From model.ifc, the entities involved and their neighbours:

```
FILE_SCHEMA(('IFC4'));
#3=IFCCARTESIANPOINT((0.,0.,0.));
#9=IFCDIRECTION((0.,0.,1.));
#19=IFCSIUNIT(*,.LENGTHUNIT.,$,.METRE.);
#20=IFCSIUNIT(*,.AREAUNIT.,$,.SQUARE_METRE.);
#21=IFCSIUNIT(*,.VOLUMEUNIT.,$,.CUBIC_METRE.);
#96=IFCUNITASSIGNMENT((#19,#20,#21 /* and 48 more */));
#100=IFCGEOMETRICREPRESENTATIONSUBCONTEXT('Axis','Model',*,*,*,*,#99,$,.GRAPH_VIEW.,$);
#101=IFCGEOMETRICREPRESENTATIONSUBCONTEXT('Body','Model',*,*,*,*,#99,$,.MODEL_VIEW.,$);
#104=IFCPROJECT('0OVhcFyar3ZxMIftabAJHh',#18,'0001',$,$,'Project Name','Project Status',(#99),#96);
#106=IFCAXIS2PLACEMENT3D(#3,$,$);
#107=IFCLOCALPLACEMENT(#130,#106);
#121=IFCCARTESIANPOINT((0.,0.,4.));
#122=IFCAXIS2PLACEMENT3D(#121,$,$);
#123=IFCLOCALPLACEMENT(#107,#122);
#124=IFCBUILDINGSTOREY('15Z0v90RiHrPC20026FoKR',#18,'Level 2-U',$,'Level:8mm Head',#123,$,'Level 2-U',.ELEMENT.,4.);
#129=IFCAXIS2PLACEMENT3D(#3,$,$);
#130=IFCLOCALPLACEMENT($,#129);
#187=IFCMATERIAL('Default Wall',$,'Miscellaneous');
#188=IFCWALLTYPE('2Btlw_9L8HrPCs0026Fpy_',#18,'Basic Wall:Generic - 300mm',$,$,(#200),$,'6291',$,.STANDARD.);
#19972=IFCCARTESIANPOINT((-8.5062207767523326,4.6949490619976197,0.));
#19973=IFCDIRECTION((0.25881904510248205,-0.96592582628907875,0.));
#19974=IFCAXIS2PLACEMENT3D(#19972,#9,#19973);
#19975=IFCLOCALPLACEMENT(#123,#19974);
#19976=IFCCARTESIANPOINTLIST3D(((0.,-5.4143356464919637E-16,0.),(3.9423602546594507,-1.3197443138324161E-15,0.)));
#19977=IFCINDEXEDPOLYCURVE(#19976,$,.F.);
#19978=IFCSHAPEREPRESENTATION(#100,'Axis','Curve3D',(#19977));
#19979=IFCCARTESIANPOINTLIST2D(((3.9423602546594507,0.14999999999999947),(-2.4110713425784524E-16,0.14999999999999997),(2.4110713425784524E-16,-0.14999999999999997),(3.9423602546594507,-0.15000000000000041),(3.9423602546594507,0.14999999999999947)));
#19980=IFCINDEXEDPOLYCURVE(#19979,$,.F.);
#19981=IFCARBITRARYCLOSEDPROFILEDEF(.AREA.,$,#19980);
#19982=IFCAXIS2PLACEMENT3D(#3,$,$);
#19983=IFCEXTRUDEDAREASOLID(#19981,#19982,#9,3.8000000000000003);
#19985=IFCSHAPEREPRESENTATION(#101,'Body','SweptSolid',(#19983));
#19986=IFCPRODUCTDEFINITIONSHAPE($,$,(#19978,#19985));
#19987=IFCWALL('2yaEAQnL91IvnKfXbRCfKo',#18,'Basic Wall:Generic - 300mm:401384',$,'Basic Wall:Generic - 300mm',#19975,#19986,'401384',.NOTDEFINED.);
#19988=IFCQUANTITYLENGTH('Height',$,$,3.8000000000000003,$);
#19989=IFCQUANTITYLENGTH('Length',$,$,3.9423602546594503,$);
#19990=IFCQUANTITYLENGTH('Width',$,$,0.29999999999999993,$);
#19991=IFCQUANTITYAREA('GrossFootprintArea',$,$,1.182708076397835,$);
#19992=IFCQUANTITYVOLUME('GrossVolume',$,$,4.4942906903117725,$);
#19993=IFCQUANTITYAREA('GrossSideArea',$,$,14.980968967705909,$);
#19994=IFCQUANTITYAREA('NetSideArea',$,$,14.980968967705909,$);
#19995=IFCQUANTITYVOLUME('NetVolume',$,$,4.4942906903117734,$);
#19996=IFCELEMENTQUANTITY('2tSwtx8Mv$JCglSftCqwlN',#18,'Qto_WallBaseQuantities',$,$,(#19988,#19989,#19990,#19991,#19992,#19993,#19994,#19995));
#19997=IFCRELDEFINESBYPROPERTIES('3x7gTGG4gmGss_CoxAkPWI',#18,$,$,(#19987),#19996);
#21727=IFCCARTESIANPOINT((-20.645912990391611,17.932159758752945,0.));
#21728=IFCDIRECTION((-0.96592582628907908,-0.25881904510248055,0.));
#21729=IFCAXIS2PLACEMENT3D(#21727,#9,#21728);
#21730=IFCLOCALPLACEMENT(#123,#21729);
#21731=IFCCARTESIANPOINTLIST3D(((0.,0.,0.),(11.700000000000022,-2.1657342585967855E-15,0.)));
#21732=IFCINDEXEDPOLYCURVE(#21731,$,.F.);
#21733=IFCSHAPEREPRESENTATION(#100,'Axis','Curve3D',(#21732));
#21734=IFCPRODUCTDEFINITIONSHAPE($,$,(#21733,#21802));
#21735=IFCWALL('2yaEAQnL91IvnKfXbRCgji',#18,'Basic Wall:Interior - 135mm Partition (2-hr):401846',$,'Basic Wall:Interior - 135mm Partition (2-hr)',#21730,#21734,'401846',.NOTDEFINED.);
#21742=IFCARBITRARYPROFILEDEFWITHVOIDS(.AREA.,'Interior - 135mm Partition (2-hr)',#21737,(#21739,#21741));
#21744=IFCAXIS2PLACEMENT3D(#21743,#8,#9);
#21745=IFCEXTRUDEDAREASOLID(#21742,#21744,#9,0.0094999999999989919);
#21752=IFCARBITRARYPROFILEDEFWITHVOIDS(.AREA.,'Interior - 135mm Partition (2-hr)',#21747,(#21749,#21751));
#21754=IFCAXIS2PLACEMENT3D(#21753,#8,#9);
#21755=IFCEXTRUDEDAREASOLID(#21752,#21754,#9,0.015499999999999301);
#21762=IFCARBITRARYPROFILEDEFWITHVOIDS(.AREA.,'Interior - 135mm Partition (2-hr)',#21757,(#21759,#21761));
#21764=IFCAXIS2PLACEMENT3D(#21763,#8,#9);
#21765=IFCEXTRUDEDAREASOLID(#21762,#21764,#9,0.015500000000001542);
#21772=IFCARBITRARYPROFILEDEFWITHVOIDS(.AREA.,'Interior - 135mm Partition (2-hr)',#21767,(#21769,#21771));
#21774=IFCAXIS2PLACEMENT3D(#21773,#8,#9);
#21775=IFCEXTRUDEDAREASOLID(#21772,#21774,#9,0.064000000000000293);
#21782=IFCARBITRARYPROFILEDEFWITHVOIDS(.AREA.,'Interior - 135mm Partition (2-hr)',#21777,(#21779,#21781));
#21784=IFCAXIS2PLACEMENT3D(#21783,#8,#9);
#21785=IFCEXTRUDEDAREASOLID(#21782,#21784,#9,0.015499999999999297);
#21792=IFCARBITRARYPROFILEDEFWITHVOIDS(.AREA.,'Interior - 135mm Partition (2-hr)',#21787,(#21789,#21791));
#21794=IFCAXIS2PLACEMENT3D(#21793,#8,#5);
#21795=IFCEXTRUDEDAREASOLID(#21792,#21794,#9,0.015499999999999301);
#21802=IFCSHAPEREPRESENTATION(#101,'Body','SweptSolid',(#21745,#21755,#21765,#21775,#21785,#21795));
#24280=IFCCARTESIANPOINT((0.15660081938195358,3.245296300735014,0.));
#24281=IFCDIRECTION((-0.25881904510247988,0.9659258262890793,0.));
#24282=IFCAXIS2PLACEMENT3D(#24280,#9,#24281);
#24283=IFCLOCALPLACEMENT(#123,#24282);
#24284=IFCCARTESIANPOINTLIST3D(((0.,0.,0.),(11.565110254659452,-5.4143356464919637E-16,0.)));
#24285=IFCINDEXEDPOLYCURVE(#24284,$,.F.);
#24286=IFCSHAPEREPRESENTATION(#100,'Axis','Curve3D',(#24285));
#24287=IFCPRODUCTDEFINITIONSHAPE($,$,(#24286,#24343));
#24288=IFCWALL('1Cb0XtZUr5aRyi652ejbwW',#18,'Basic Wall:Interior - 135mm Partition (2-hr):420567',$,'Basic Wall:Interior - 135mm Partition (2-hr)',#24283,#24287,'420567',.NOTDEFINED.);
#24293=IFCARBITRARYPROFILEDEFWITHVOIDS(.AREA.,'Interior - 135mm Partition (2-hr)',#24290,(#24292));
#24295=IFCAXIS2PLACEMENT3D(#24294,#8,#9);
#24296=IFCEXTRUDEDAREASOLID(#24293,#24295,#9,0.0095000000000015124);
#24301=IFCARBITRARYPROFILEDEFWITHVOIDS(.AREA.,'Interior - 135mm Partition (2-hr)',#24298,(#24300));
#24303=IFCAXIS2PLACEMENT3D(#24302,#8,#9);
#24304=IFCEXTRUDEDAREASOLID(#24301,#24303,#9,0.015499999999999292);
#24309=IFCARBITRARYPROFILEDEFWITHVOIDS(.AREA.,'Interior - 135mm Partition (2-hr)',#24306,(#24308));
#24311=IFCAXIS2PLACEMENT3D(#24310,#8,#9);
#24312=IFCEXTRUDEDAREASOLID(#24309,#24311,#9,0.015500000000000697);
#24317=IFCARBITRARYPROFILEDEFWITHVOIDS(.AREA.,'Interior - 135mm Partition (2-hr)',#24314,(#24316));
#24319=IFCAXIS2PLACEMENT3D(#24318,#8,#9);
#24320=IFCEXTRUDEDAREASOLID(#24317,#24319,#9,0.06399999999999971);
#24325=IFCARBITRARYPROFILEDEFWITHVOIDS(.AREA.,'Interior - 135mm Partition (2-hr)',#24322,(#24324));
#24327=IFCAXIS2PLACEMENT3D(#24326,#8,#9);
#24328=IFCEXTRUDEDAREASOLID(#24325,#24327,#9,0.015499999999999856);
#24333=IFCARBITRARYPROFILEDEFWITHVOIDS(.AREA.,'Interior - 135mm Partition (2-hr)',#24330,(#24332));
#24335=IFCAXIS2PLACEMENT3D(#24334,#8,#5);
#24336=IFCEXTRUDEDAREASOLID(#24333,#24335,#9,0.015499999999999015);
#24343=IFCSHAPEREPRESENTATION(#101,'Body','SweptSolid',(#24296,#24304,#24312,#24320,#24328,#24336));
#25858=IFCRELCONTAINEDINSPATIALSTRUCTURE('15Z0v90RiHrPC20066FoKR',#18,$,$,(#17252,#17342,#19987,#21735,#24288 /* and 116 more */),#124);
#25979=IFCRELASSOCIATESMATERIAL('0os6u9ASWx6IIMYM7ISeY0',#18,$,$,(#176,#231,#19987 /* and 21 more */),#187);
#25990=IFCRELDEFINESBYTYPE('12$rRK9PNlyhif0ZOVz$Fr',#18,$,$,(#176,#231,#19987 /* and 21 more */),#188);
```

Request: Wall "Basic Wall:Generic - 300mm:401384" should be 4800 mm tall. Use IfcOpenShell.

```python
import ifcopenshell
import ifcopenshell.api.pset
import ifcopenshell.geom
import ifcopenshell.util.element
import ifcopenshell.util.representation
import ifcopenshell.util.shape
import ifcopenshell.util.unit

model = ifcopenshell.open("model.ifc")
unit_scale = ifcopenshell.util.unit.calculate_unit_scale(model)
area_scale = ifcopenshell.util.unit.calculate_unit_scale(model, "AREAUNIT")
volume_scale = ifcopenshell.util.unit.calculate_unit_scale(model, "VOLUMEUNIT")
settings = ifcopenshell.geom.settings()


def volume(element):
    """Net volume in cubic metres, openings subtracted."""
    shape = ifcopenshell.geom.create_shape(settings, element)
    return ifcopenshell.util.shape.get_volume(shape.geometry)


wall = model.by_id(19987)
before = volume(wall)

body = ifcopenshell.util.representation.get_representation(wall, "Model", "Body")
solid = body.Items[0]
old_height = solid.Depth
solid.Depth = 4.8
after = volume(wall)
thickness = 0.3  # wall thickness in metres

# Update the stored height, areas and volumes.
qto = model.by_id(ifcopenshell.util.element.get_pset(wall, "Qto_WallBaseQuantities", should_inherit=False)["id"])
ifcopenshell.api.pset.edit_qto(model, qto=qto, properties={
    "Height": solid.Depth,
    "GrossVolume": ifcopenshell.util.element.get_pset(wall, "Qto_WallBaseQuantities", "GrossVolume") * solid.Depth / old_height,
    "GrossSideArea": ifcopenshell.util.element.get_pset(wall, "Qto_WallBaseQuantities", "GrossSideArea") * solid.Depth / old_height,
    "NetSideArea": after / thickness / area_scale,
    "NetVolume": after / volume_scale,
})

print(f"height {old_height:g} -> {solid.Depth:g}, volume {before:.3f} -> {after:.3f} m3")

model.write("model_rev.ifc")
```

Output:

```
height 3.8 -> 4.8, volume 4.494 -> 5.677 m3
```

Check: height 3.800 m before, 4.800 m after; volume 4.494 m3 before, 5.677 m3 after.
